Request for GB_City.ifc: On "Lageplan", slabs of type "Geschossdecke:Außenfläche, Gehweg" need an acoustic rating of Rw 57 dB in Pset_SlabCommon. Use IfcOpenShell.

First a look at what the model holds.

```python
import ifcopenshell
import ifcopenshell.util.element

model = ifcopenshell.open("GB_City.ifc")
print(model.schema)
storey = next(s for s in model.by_type("IfcBuildingStorey") if s.Name == "Lageplan")
slabs = [e for e in ifcopenshell.util.element.get_decomposition(storey) if e.is_a("IfcSlab")]
seen = {}
for e in slabs:
    element_type = ifcopenshell.util.element.get_type(e)
    key = (element_type.Name if element_type != e and element_type else None, ifcopenshell.util.element.get_pset(e, "Pset_SlabCommon", "AcousticRating"))
    seen[key] = seen.get(key, 0) + 1
for (name, value), count in sorted(seen.items(), key=str):
    print(count, "x", name, "|", value)
```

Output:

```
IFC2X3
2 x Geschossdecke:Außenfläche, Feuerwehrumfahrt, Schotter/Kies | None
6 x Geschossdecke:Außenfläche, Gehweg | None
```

```python
import ifcopenshell
import ifcopenshell.api.pset
import ifcopenshell.util.element

model = ifcopenshell.open("GB_City.ifc")

storey = next(s for s in model.by_type("IfcBuildingStorey") if s.Name == "Lageplan")
slabs = [e for e in ifcopenshell.util.element.get_decomposition(storey) if e.is_a("IfcSlab")]

count = 0
for e in slabs:
    element_type = ifcopenshell.util.element.get_type(e)
    if element_type in (None, e) or element_type.Name != "Geschossdecke:Außenfläche, Gehweg":
        continue
    # add_pset returns the element's existing set when there is one.
    pset = ifcopenshell.api.pset.add_pset(model, product=e, name="Pset_SlabCommon")
    ifcopenshell.api.pset.edit_pset(model, pset=pset, properties={"AcousticRating": "Rw 57 dB"})
    count += 1

print(count, "slabs updated")

model.write("GB_City_updated.ifc")
```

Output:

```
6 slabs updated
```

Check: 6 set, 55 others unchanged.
